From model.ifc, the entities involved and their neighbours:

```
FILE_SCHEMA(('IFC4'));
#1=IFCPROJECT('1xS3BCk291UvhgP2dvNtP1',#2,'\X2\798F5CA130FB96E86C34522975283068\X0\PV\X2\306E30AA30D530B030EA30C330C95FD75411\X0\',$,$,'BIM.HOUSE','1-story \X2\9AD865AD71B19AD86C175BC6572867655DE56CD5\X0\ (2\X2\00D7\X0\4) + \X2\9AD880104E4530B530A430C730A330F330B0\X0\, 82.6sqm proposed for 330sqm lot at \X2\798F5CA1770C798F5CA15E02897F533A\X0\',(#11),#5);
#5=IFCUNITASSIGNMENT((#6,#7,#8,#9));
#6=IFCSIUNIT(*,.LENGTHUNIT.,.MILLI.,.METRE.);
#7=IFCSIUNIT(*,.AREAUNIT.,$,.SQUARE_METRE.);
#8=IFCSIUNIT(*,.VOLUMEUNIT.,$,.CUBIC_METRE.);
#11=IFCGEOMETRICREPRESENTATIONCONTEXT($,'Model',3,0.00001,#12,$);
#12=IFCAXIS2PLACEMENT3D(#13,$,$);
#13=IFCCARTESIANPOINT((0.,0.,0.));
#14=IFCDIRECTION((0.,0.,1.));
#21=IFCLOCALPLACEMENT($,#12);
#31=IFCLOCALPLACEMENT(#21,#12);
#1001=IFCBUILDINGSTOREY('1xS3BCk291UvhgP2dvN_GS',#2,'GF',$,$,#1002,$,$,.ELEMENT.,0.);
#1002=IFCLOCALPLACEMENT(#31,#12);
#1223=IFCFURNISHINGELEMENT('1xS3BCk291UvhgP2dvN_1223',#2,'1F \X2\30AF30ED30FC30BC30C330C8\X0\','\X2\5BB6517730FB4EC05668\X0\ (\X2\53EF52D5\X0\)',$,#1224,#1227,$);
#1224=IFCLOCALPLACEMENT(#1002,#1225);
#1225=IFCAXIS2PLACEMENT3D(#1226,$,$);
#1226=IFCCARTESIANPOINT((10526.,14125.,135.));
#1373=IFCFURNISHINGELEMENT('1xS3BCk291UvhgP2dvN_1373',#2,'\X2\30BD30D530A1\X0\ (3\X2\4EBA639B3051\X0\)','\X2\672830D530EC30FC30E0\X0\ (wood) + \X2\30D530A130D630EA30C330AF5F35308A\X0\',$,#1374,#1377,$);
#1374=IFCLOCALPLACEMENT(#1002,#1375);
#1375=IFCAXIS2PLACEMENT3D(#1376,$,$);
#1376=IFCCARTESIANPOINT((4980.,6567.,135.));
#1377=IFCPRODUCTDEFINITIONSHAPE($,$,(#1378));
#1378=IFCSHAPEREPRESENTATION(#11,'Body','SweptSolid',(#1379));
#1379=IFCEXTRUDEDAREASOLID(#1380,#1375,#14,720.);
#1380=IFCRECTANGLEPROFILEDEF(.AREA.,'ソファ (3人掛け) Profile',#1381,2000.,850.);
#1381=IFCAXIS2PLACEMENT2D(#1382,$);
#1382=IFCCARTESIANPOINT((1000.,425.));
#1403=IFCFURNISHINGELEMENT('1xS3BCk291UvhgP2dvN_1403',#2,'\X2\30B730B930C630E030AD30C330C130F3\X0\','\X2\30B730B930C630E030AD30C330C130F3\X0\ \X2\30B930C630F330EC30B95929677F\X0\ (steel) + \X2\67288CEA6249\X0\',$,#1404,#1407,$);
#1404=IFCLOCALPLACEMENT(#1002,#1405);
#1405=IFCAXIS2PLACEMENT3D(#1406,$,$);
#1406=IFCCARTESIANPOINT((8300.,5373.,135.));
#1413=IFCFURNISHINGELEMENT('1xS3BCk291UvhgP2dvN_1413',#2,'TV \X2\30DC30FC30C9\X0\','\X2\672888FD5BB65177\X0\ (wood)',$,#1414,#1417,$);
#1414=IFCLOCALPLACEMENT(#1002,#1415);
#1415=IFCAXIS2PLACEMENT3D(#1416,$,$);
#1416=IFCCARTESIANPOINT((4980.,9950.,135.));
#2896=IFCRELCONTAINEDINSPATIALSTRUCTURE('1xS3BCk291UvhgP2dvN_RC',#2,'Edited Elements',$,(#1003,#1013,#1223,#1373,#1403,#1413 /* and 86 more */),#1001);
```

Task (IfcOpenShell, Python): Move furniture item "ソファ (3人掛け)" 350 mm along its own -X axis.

```python
import ifcopenshell
import ifcopenshell.api.geometry
import ifcopenshell.util.placement
import ifcopenshell.util.unit

model = ifcopenshell.open("model.ifc")
unit_scale = ifcopenshell.util.unit.calculate_unit_scale(model)

item = model.by_guid("1xS3BCk291UvhgP2dvN_1373")
matrix = ifcopenshell.util.placement.get_local_placement(item.ObjectPlacement)
matrix[:3, 3] -= matrix[:3, 0] * 0.35 / unit_scale
ifcopenshell.api.geometry.edit_object_placement(model, product=item, matrix=matrix, is_si=False)

print(ifcopenshell.util.placement.get_local_placement(item.ObjectPlacement).round(3) + 0.0)

model.write("model_updated.ifc")
```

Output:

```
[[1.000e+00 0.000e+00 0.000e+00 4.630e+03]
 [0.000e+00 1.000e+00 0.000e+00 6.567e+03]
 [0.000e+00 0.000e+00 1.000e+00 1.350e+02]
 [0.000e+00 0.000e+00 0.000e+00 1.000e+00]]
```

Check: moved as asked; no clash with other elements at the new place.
